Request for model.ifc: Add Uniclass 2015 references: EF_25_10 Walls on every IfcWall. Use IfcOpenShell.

First a look at what the model holds.

```python
import ifcopenshell

model = ifcopenshell.open("model.ifc")
print(model.schema)
print("classifications:", [c.Name for c in model.by_type("IfcClassification")])
for ifc_class in ("IfcDoor", "IfcRoof", "IfcStair", "IfcWall", "IfcWindow"):
    print(ifc_class, len(model.by_type(ifc_class)))
```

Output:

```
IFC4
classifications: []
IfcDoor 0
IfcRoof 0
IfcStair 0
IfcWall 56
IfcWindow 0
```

```python
import ifcopenshell
import ifcopenshell.api.classification

model = ifcopenshell.open("model.ifc")

system = ifcopenshell.api.classification.add_classification(model, classification="Uniclass 2015")

codes = {
    "IfcWall": ("EF_25_10", "Walls"),
}
for ifc_class, (code, name) in codes.items():
    products = model.by_type(ifc_class)
    ifcopenshell.api.classification.add_reference(
        model, products=products, classification=system, identification=code, name=name
    )
    print(code, len(products))

model.write("model_edited.ifc")
```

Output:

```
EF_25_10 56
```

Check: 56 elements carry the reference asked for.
